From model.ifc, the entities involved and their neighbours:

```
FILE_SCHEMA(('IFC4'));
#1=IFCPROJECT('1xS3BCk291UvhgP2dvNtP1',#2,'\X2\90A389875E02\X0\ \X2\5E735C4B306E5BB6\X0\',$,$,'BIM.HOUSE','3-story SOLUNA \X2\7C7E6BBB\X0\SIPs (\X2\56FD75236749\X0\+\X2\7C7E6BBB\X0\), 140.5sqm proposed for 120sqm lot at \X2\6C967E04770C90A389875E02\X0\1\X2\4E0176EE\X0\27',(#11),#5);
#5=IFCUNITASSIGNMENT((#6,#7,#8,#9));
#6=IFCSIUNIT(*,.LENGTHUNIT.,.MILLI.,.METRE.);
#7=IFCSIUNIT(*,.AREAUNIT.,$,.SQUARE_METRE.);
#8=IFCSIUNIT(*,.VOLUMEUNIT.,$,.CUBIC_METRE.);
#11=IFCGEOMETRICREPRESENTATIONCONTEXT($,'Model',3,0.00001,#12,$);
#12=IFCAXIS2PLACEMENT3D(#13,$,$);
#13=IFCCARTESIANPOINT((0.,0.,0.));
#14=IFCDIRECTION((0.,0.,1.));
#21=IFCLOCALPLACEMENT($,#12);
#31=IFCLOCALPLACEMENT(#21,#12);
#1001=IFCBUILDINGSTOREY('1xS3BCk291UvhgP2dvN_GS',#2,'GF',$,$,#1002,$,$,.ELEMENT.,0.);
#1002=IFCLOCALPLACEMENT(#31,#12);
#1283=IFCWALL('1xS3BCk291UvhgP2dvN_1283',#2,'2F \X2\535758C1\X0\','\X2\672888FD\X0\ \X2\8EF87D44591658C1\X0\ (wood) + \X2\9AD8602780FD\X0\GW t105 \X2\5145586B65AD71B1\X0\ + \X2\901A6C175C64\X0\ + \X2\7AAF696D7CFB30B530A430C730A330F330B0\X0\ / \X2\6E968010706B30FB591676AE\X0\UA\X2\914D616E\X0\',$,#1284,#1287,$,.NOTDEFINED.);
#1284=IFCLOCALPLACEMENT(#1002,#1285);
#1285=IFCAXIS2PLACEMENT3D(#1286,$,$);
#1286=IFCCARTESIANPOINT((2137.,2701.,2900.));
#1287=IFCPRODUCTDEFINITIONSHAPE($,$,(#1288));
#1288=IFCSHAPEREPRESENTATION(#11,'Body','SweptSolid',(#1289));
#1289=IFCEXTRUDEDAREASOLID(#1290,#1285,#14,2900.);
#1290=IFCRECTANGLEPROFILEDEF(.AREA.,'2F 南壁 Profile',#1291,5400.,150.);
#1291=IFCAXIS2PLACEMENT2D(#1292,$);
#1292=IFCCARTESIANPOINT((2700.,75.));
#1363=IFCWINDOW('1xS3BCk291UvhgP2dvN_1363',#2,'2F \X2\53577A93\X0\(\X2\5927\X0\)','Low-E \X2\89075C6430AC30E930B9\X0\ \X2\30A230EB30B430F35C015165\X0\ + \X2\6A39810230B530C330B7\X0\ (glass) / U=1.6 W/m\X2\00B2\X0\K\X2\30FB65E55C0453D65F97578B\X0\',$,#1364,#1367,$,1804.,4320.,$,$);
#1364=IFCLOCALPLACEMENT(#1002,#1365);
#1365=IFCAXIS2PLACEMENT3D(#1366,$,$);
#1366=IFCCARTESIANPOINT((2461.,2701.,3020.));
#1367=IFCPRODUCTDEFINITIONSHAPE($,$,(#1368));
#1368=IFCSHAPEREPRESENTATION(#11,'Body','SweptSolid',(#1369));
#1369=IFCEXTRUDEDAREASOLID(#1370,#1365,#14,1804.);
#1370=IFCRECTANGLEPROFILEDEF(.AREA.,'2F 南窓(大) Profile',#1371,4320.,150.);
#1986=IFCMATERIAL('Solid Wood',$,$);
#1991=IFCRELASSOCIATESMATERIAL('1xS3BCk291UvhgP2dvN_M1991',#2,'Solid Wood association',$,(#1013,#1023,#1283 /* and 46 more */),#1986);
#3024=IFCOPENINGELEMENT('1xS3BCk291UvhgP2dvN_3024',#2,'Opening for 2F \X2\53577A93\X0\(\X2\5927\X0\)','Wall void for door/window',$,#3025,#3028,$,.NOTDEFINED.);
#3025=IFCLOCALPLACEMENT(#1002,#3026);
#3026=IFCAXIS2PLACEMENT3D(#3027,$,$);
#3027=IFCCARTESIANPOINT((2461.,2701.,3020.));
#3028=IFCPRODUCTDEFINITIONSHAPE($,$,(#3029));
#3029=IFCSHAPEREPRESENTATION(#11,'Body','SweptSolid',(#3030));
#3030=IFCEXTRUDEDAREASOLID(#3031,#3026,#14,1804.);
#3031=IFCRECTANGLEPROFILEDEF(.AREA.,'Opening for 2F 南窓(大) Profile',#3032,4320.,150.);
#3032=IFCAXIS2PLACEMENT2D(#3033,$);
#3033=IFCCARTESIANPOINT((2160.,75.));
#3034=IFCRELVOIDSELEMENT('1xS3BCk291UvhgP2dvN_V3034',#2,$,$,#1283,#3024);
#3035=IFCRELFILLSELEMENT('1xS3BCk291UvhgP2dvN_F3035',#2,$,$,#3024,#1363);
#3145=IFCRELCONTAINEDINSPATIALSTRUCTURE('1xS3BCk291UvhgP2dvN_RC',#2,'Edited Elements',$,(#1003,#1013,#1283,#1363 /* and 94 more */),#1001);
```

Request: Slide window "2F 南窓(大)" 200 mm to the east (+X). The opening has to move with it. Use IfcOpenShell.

```python
import ifcopenshell
import ifcopenshell.api.geometry
import ifcopenshell.util.placement
import ifcopenshell.util.unit

model = ifcopenshell.open("model.ifc")
unit_scale = ifcopenshell.util.unit.calculate_unit_scale(model)

window = model.by_guid("1xS3BCk291UvhgP2dvN_1363")
opening = window.FillsVoids[0].RelatingOpeningElement
wall = opening.VoidsElements[0].RelatingBuildingElement

wall_matrix = ifcopenshell.util.placement.get_local_placement(wall.ObjectPlacement)
shift = wall_matrix[:3, 0] * 0.2 / unit_scale
before = ifcopenshell.util.placement.get_local_placement(window.ObjectPlacement)[:3, 3].copy()

# The window is not placed relative to its opening, so move both.
for product in (opening, window):
    matrix = ifcopenshell.util.placement.get_local_placement(product.ObjectPlacement)
    matrix[:3, 3] += shift
    ifcopenshell.api.geometry.edit_object_placement(model, product=product, matrix=matrix, is_si=False)

after = ifcopenshell.util.placement.get_local_placement(window.ObjectPlacement)[:3, 3]
print("window moved by", (after - before).round(3) + 0.0)

model.write("model_v2.ifc")
```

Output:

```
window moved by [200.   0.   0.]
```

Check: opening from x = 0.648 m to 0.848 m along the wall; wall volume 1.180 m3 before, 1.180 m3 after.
